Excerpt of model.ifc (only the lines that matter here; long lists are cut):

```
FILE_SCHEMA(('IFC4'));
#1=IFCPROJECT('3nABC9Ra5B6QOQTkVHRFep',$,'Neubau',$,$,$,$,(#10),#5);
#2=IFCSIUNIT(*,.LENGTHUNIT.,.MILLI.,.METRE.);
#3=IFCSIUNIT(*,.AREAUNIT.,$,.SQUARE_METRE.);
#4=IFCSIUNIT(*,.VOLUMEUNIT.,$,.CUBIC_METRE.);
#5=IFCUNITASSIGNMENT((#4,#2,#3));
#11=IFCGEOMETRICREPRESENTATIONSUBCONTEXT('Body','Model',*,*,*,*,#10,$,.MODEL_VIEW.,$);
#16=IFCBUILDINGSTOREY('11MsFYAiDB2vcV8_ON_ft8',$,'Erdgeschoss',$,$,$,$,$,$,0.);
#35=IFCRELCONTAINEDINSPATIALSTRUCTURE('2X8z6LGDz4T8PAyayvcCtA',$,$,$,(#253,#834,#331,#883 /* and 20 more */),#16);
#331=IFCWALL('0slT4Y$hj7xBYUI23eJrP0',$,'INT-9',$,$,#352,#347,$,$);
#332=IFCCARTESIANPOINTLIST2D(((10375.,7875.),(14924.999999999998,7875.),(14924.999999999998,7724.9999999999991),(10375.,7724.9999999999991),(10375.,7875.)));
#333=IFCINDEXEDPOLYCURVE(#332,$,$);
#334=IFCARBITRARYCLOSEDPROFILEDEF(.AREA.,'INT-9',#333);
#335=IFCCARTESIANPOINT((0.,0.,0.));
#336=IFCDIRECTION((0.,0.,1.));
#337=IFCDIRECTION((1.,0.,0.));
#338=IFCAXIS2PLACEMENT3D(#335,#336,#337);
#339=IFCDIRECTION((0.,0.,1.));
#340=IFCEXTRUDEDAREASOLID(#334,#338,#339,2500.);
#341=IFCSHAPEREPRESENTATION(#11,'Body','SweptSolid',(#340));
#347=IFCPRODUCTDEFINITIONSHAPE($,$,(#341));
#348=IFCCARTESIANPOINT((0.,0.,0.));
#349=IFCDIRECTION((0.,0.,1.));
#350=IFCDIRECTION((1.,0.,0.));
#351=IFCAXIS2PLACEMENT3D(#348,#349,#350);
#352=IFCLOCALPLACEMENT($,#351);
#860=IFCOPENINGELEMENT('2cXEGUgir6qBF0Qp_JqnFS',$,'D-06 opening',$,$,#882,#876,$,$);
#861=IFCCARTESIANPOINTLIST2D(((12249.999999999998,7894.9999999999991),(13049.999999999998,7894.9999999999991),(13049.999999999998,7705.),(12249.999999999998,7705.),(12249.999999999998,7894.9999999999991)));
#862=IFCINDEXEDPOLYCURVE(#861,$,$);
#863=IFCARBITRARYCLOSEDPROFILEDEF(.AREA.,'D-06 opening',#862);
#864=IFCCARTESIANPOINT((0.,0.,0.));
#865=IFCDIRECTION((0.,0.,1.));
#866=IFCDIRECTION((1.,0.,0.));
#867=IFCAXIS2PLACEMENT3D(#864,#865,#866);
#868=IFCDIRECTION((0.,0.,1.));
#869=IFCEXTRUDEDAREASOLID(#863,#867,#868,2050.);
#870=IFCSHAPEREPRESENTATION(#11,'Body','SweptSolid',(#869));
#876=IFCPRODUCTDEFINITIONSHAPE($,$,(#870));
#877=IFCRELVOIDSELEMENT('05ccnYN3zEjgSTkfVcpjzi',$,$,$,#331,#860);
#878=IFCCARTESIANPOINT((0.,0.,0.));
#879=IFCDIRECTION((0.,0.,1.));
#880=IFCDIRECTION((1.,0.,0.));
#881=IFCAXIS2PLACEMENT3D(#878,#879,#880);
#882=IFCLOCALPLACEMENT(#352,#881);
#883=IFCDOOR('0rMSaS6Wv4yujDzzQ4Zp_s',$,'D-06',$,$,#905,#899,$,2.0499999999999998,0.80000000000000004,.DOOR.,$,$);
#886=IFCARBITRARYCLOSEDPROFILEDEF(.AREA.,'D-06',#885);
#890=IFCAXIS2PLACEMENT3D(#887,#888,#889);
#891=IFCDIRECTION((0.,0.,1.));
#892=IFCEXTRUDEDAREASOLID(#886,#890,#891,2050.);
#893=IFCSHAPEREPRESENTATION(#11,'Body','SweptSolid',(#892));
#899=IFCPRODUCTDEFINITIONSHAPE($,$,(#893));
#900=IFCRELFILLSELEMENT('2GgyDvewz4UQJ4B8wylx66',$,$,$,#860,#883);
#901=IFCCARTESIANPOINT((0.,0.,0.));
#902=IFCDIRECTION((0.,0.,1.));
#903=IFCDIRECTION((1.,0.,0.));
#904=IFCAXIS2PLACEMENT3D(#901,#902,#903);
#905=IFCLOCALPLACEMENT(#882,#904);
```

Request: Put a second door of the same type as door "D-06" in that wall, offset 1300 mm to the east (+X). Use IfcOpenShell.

```python
import ifcopenshell
import ifcopenshell.api.feature
import ifcopenshell.api.geometry
import ifcopenshell.api.root
import ifcopenshell.geom
import ifcopenshell.util.element
import ifcopenshell.util.placement
import ifcopenshell.util.shape
import ifcopenshell.util.unit

model = ifcopenshell.open("model.ifc")
unit_scale = ifcopenshell.util.unit.calculate_unit_scale(model)
settings = ifcopenshell.geom.settings()


def volume(element):
    """Net volume in cubic metres, openings subtracted."""
    shape = ifcopenshell.geom.create_shape(settings, element)
    return ifcopenshell.util.shape.get_volume(shape.geometry)


door = model.by_guid("0rMSaS6Wv4yujDzzQ4Zp_s")
opening = door.FillsVoids[0].RelatingOpeningElement
wall = opening.VoidsElements[0].RelatingBuildingElement
before = volume(wall)
shift = ifcopenshell.util.placement.get_local_placement(wall.ObjectPlacement)[:3, 0] * 1.3 / unit_scale

# copy_class copies the void relationship, type, container and properties, but no geometry.
new_opening = ifcopenshell.api.root.copy_class(model, product=opening)
new_opening.Representation = ifcopenshell.util.element.copy_deep(
    model, opening.Representation, exclude=["IfcGeometricRepresentationContext", "IfcRepresentationMap"]
)
new_door = ifcopenshell.api.root.copy_class(model, product=door)
new_door.Representation = ifcopenshell.util.element.copy_deep(
    model, door.Representation, exclude=["IfcGeometricRepresentationContext", "IfcRepresentationMap"]
)
ifcopenshell.api.feature.add_filling(model, opening=new_opening, element=new_door)

for old, new in ((opening, new_opening), (door, new_door)):
    matrix = ifcopenshell.util.placement.get_local_placement(old.ObjectPlacement)
    matrix[:3, 3] += shift
    ifcopenshell.api.geometry.edit_object_placement(model, product=new, matrix=matrix, is_si=False)

after = volume(wall)

print(f"wall volume {before:.3f} -> {after:.3f} m3")

model.write("model-out.ifc")
```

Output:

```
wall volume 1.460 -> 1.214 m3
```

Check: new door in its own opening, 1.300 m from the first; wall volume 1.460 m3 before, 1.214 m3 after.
